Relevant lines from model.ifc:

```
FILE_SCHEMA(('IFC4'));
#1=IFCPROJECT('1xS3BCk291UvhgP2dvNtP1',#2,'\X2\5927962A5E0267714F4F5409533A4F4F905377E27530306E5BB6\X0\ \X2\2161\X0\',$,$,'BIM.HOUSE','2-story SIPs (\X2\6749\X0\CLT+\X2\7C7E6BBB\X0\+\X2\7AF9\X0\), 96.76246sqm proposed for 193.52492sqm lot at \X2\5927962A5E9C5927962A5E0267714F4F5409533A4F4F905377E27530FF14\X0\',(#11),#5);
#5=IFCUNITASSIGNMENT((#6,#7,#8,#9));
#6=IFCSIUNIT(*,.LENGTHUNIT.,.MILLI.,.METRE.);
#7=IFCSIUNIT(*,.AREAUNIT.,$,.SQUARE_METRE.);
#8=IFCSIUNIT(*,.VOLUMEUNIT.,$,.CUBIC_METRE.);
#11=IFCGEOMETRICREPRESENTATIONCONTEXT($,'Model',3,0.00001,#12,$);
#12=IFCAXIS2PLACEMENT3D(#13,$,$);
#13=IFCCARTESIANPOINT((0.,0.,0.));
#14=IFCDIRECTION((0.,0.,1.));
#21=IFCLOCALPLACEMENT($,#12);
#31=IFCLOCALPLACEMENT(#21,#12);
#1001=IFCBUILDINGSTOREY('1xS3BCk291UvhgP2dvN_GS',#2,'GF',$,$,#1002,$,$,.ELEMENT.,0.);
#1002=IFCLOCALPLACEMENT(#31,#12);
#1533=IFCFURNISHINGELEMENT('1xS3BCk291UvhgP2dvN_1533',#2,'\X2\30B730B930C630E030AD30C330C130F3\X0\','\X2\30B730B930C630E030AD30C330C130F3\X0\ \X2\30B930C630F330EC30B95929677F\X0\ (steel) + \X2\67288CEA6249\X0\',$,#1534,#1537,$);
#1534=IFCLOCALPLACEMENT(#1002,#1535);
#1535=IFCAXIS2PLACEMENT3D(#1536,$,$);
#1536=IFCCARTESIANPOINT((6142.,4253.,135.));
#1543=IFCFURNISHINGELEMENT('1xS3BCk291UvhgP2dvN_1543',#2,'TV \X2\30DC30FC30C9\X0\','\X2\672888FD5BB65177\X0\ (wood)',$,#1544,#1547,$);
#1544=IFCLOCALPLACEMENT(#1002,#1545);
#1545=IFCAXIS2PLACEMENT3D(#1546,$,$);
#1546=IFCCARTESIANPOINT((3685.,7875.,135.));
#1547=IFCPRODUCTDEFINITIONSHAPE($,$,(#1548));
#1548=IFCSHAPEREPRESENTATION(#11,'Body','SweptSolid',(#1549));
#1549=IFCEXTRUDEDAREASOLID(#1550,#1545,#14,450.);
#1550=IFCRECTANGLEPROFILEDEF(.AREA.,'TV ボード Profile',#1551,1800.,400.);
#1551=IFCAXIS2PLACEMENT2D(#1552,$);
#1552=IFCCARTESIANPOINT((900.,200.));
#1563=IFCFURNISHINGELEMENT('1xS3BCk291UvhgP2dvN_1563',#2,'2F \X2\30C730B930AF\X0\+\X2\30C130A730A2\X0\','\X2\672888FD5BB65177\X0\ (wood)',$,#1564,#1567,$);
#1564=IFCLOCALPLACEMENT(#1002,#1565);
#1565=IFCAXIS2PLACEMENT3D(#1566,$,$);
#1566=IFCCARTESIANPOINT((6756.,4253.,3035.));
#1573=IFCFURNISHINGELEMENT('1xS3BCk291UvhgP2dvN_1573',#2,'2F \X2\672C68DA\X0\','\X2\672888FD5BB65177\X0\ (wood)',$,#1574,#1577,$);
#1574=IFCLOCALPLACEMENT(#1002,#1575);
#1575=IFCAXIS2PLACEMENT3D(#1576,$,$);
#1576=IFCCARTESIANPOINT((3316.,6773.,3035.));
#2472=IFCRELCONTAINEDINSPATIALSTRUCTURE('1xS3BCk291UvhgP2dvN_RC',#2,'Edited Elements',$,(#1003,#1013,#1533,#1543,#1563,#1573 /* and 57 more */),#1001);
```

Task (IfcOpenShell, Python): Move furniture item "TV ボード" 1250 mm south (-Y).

```python
import ifcopenshell
import ifcopenshell.api.geometry
import ifcopenshell.util.placement
import ifcopenshell.util.unit

model = ifcopenshell.open("model.ifc")
unit_scale = ifcopenshell.util.unit.calculate_unit_scale(model)

item = model.by_guid("1xS3BCk291UvhgP2dvN_1543")
matrix = ifcopenshell.util.placement.get_local_placement(item.ObjectPlacement)
matrix[1, 3] -= 1.25 / unit_scale
ifcopenshell.api.geometry.edit_object_placement(model, product=item, matrix=matrix, is_si=False)

print(ifcopenshell.util.placement.get_local_placement(item.ObjectPlacement).round(3) + 0.0)

model.write("model-out.ifc")
```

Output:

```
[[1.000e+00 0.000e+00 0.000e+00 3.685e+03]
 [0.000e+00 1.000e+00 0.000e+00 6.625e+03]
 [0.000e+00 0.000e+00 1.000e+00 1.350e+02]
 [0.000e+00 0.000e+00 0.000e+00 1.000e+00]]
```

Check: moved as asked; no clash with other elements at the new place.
